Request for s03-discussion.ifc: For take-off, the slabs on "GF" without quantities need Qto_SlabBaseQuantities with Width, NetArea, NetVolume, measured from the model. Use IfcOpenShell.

First a look at what the model holds.

```python
import ifcopenshell
import ifcopenshell.util.element
import ifcopenshell.util.unit

model = ifcopenshell.open("s03-discussion.ifc")
print(model.schema)
for unit_type in ("LENGTHUNIT", "AREAUNIT", "VOLUMEUNIT"):
    print(unit_type, ifcopenshell.util.unit.calculate_unit_scale(model, unit_type))
storey = next(s for s in model.by_type("IfcBuildingStorey") if s.Name == "GF")
slabs = [e for e in ifcopenshell.util.element.get_decomposition(storey) if e.is_a("IfcSlab")]
for e in sorted(slabs, key=lambda e: e.id()):
    print(e.id(), e.is_a(), e.Name, list(ifcopenshell.util.element.get_psets(e, qtos_only=True)), sep=" | ")
```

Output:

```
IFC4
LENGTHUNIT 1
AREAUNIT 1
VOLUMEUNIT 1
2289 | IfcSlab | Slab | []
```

```python
import ifcopenshell
import ifcopenshell.api.pset
import ifcopenshell.geom
import ifcopenshell.util.element
import ifcopenshell.util.shape
import ifcopenshell.util.unit

model = ifcopenshell.open("s03-discussion.ifc")
unit_scale = ifcopenshell.util.unit.calculate_unit_scale(model)
area_scale = ifcopenshell.util.unit.calculate_unit_scale(model, "AREAUNIT")
volume_scale = ifcopenshell.util.unit.calculate_unit_scale(model, "VOLUMEUNIT")
settings = ifcopenshell.geom.settings()

storey = next(s for s in model.by_type("IfcBuildingStorey") if s.Name == "GF")
slabs = [e for e in ifcopenshell.util.element.get_decomposition(storey) if e.is_a("IfcSlab")]

for e in sorted(slabs, key=lambda e: e.id()):
    if ifcopenshell.util.element.get_psets(e, qtos_only=True, should_inherit=False):
        continue
    # Geometry comes back in metres, in the element's own axes.
    shape = ifcopenshell.geom.create_shape(settings, e)
    values = {
        "Width": ifcopenshell.util.shape.get_z(shape.geometry) / unit_scale,
        "NetArea": ifcopenshell.util.shape.get_footprint_area(shape.geometry) / area_scale,
        "NetVolume": ifcopenshell.util.shape.get_volume(shape.geometry) / volume_scale,
    }
    qto = ifcopenshell.api.pset.add_qto(model, product=e, name="Qto_SlabBaseQuantities")
    ifcopenshell.api.pset.edit_qto(model, qto=qto, properties=values)
    print(e.id(), {k: round(v, 3) for k, v in values.items()})

model.write("s03-discussion_updated.ifc")
```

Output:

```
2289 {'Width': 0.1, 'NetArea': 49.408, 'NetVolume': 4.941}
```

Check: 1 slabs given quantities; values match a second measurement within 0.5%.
